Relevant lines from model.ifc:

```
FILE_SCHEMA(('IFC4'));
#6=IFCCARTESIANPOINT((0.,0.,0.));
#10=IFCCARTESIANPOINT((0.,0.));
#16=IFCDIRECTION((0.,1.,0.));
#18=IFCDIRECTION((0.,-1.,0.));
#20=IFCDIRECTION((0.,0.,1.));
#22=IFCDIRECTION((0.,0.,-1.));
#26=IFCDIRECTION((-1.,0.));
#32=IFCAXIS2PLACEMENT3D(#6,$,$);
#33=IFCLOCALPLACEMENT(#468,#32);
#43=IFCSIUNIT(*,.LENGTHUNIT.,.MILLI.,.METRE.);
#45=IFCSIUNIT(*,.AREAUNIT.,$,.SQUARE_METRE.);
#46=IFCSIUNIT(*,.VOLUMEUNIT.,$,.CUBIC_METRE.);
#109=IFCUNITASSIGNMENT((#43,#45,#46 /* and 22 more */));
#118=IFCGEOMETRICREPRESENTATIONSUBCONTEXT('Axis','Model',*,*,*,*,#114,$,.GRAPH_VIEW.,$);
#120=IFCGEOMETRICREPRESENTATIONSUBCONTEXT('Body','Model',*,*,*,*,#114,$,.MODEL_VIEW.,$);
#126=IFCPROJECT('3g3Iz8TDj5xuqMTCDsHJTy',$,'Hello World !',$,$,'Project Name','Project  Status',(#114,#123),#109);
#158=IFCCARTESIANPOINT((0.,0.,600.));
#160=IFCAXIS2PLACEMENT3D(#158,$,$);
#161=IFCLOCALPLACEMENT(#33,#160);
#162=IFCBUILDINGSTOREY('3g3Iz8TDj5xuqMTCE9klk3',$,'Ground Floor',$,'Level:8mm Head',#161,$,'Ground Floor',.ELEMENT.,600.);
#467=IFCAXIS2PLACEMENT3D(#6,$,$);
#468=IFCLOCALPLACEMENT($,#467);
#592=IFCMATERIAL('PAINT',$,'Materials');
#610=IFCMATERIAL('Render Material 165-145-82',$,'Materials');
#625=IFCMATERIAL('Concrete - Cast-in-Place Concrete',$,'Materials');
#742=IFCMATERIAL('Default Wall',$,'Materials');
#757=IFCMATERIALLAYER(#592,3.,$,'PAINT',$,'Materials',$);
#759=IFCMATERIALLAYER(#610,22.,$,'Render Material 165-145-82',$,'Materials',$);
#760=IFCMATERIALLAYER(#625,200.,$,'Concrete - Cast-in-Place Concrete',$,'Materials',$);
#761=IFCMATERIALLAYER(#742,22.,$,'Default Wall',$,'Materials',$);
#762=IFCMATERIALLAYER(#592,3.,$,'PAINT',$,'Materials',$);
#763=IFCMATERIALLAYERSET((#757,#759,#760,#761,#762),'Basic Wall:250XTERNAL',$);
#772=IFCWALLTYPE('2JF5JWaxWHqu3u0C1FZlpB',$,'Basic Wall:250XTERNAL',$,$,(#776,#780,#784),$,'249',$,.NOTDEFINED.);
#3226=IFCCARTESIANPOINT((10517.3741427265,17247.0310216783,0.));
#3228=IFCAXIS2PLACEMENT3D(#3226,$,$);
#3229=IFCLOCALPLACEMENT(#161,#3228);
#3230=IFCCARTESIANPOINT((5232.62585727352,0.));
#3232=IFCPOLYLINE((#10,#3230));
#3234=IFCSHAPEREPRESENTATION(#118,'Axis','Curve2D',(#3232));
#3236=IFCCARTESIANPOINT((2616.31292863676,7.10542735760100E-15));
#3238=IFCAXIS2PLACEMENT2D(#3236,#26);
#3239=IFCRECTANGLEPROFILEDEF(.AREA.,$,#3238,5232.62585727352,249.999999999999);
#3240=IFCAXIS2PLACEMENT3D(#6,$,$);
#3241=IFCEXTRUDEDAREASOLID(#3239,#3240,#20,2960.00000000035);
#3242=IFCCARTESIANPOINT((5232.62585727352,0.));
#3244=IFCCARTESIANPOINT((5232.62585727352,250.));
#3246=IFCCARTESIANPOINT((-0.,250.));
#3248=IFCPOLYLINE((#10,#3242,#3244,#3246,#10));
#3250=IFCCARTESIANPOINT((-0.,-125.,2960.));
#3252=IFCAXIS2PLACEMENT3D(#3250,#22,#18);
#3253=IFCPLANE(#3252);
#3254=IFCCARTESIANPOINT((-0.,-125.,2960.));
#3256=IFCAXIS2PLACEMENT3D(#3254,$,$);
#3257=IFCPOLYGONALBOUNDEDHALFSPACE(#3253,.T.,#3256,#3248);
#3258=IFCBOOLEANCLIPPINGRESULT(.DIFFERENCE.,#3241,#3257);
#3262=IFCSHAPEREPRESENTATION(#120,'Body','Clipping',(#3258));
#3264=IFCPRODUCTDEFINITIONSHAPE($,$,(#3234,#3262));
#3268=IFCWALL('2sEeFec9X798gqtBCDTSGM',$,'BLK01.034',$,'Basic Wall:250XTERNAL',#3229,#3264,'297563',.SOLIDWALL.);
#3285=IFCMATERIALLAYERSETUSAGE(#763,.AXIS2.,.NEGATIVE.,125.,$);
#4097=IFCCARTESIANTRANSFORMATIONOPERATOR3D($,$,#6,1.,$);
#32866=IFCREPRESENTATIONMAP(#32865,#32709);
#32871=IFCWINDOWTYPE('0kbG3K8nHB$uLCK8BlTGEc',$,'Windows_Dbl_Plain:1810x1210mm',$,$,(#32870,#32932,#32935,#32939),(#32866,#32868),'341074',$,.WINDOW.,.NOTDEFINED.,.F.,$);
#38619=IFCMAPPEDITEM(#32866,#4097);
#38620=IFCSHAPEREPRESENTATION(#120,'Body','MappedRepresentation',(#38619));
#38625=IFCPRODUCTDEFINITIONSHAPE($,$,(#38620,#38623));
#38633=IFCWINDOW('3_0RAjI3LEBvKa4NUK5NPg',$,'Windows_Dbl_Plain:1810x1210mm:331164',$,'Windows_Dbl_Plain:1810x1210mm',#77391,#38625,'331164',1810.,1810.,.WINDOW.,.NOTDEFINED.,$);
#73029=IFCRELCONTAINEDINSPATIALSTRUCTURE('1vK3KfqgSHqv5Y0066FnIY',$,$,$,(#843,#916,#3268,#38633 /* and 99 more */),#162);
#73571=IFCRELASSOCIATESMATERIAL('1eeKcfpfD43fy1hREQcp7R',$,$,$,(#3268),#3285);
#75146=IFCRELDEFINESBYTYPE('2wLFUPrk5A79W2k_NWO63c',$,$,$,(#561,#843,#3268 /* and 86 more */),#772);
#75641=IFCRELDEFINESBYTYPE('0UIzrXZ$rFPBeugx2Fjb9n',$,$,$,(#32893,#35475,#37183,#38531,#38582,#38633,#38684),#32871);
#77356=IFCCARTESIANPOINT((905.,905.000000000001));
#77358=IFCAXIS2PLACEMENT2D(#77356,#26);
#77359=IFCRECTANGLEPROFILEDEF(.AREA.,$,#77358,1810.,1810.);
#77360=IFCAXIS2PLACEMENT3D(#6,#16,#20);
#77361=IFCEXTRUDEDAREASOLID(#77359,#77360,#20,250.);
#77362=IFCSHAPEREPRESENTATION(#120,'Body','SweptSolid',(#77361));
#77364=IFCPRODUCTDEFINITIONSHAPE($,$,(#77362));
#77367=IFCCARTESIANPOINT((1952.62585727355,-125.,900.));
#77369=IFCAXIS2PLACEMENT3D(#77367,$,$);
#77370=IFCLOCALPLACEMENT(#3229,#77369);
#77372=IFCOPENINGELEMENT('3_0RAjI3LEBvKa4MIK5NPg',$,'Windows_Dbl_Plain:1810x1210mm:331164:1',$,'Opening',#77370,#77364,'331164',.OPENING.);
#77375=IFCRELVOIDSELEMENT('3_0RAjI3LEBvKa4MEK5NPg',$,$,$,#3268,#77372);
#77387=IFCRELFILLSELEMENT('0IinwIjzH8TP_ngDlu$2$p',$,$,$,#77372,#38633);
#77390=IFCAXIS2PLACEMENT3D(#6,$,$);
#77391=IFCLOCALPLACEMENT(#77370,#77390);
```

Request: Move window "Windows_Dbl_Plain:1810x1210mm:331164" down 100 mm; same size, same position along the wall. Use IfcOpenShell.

```python
import numpy as np
import ifcopenshell
import ifcopenshell.api.geometry
import ifcopenshell.util.placement
import ifcopenshell.util.unit

model = ifcopenshell.open("model.ifc")
unit_scale = ifcopenshell.util.unit.calculate_unit_scale(model)

window = model.by_guid("3_0RAjI3LEBvKa4NUK5NPg")
opening = window.FillsVoids[0].RelatingOpeningElement
dz = -0.1 / unit_scale

shift = np.array([0.0, 0.0, dz])
# The window is placed relative to its opening, so it follows when the opening moves.
matrix = ifcopenshell.util.placement.get_local_placement(opening.ObjectPlacement)
matrix[:3, 3] += shift
ifcopenshell.api.geometry.edit_object_placement(
    model, product=opening, matrix=matrix, is_si=False, should_transform_children=True
)

print(f"moved by {dz * unit_scale:+.3f} m")

model.write("model-out.ifc")
```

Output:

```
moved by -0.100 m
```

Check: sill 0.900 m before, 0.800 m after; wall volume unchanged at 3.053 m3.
